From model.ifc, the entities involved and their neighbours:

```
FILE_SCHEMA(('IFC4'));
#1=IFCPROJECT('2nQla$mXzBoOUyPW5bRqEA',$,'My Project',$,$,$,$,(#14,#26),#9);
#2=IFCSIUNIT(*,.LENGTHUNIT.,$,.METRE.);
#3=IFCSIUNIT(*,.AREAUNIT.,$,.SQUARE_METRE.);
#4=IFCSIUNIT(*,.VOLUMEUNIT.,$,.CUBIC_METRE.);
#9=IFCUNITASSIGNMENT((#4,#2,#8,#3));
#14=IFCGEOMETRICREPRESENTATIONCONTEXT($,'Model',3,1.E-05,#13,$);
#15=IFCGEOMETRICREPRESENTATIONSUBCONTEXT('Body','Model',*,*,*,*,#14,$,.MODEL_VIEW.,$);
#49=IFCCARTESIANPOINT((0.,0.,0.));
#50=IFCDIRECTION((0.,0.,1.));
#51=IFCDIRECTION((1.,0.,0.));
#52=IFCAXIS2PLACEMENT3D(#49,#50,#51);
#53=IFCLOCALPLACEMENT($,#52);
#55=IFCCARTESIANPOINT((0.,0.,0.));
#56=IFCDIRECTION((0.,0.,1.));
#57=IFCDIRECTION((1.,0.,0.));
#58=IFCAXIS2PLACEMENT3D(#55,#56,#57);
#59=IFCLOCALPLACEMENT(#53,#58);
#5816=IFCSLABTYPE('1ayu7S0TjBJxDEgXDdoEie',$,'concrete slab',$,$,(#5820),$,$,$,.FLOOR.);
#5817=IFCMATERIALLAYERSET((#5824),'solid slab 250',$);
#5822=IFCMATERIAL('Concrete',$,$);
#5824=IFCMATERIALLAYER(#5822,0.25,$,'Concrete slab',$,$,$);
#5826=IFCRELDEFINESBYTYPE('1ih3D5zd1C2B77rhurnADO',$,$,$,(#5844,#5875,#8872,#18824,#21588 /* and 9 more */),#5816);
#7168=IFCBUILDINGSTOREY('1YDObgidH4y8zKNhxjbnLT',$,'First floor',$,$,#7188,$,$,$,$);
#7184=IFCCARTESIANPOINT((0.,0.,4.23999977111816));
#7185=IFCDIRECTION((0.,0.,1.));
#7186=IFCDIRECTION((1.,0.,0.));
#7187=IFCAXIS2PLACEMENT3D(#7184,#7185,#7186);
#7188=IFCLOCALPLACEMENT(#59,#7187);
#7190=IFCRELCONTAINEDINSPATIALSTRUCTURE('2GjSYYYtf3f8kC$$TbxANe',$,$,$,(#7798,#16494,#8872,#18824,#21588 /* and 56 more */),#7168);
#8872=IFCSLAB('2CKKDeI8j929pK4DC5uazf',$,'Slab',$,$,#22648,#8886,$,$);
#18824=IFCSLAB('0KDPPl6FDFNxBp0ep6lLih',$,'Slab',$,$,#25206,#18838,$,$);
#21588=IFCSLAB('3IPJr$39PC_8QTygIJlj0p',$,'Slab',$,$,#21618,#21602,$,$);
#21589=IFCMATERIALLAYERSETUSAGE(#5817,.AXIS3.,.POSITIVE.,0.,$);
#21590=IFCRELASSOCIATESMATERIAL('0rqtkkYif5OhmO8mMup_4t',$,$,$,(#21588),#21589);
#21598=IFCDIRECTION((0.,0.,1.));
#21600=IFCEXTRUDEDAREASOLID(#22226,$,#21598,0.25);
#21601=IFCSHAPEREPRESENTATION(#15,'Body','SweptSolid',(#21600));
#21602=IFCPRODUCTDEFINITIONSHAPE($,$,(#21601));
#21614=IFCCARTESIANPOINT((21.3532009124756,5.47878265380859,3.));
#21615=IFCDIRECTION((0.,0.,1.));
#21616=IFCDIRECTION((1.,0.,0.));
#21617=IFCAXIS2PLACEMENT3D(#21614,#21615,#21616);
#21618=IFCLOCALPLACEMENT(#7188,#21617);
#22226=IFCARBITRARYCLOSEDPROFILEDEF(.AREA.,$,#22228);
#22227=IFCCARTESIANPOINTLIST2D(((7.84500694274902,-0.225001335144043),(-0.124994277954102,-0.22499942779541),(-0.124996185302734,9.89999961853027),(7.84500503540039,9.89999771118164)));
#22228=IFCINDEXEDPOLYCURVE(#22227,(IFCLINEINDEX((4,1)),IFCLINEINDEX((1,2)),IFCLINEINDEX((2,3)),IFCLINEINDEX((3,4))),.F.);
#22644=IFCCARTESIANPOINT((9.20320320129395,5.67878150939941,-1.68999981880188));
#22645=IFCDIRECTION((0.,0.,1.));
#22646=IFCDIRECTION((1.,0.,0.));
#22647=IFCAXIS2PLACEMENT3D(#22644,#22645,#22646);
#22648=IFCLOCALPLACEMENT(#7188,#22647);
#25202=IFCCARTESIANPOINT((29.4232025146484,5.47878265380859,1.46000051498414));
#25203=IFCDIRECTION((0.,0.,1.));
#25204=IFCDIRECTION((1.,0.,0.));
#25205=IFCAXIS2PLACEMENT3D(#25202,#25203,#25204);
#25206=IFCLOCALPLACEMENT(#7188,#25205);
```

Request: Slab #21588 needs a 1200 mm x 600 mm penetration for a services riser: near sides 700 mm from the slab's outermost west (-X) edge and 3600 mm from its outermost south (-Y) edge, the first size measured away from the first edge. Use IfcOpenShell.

```python
import numpy as np
import ifcopenshell
import ifcopenshell.api.feature
import ifcopenshell.api.geometry
import ifcopenshell.api.root
import ifcopenshell.geom
import ifcopenshell.util.placement
import ifcopenshell.util.representation
import ifcopenshell.util.shape
import ifcopenshell.util.unit

model = ifcopenshell.open("model.ifc")
unit_scale = ifcopenshell.util.unit.calculate_unit_scale(model)
settings = ifcopenshell.geom.settings()


def volume(element):
    """Net volume in cubic metres, openings subtracted."""
    shape = ifcopenshell.geom.create_shape(settings, element)
    return ifcopenshell.util.shape.get_volume(shape.geometry)


slab = model.by_guid("3IPJr$39PC_8QTygIJlj0p")
before = volume(slab)

# Extent in the slab's own axes, in metres. The edges named are its -X and -Y sides.
slab_shape = ifcopenshell.geom.create_shape(settings, slab)
vertices = ifcopenshell.util.shape.get_vertices(slab_shape.geometry)
x_min, y_min, bottom = vertices.min(axis=0)
top = vertices[:, 2].max()

opening = ifcopenshell.api.root.create_entity(model, ifc_class="IfcOpeningElement", name="Services riser opening", predefined_type="OPENING")
context = ifcopenshell.util.representation.get_context(model, "Model", "Body", "MODEL_VIEW")
width, depth = 1.2, 0.6
outline = [(0.0, 0.0), (width, 0.0), (width, depth), (0.0, depth), (0.0, 0.0)]
# Overshoot both faces by 50 mm so the cut is clean.
shape = ifcopenshell.api.geometry.add_slab_representation(
    model, context=context, depth=top - bottom + 0.1, polyline=outline
)
ifcopenshell.api.geometry.assign_representation(model, product=opening, representation=shape)

matrix = ifcopenshell.util.placement.get_local_placement(slab.ObjectPlacement)
matrix[:, 3] = matrix @ np.append(np.array([x_min + 0.7, y_min + 3.6, bottom - 0.05]) / unit_scale, 1.0)
ifcopenshell.api.geometry.edit_object_placement(model, product=opening, matrix=matrix, is_si=False)
ifcopenshell.api.feature.add_feature(model, feature=opening, element=slab)

after = volume(slab)

print(f"slab volume {before:.3f} -> {after:.3f} m3")

model.write("model_updated.ifc")
```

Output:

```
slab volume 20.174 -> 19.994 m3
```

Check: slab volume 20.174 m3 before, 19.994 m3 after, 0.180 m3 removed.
